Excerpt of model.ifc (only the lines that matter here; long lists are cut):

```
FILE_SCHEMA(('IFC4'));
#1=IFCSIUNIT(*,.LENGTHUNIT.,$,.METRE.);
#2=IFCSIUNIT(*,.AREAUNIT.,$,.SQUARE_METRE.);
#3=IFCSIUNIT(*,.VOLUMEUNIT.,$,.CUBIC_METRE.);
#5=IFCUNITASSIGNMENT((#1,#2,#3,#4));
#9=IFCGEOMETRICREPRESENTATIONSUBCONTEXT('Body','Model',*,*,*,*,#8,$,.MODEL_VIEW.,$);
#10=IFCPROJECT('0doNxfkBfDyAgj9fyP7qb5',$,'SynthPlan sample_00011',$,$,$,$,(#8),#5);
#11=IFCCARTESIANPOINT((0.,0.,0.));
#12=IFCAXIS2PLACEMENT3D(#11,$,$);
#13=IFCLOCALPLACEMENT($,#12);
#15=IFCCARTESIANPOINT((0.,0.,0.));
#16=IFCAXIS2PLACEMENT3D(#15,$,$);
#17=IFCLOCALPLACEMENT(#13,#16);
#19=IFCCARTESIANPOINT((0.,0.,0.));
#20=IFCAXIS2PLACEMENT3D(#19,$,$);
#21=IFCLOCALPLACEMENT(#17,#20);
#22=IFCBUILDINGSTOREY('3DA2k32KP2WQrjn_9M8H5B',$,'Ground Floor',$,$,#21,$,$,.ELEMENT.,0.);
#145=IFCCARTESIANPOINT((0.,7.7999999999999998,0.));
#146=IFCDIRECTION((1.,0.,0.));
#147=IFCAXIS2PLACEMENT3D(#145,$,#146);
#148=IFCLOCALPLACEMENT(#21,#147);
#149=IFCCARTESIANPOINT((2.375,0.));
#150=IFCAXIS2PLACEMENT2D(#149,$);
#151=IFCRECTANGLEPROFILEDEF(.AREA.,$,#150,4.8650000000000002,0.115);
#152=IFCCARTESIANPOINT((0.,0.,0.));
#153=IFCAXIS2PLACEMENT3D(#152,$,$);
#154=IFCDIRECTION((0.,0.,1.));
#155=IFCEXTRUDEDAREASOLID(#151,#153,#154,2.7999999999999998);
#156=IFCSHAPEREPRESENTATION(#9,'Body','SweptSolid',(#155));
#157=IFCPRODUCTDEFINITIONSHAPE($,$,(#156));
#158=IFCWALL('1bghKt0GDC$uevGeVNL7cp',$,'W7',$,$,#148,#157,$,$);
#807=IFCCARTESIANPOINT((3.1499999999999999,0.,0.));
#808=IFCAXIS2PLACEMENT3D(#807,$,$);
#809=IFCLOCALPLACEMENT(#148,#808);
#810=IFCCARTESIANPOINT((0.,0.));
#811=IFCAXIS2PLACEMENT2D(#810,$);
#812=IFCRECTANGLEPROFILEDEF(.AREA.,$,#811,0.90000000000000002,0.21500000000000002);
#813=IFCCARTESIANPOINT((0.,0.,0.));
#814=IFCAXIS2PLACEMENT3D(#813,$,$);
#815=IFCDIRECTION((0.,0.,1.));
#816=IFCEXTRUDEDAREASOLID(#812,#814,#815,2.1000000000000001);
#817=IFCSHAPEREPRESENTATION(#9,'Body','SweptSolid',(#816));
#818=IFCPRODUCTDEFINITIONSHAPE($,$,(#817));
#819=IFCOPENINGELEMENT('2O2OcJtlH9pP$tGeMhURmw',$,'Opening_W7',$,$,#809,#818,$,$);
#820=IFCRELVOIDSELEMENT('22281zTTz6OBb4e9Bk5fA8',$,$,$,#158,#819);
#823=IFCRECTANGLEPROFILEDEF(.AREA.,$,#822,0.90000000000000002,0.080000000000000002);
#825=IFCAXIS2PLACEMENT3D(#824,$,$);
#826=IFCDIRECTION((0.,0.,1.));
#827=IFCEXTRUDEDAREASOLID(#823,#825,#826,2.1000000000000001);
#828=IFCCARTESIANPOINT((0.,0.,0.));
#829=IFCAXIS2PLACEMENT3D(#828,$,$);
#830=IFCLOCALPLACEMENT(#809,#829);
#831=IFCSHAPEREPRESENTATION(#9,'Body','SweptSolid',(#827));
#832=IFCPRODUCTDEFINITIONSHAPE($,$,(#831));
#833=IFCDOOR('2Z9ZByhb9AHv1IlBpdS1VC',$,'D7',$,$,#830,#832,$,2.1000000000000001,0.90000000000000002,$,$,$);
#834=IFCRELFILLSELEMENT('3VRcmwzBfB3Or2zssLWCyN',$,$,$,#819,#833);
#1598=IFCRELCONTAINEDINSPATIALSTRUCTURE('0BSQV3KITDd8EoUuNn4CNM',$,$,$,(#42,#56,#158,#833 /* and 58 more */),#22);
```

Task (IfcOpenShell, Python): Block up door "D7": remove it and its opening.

```python
import ifcopenshell
import ifcopenshell.api.feature
import ifcopenshell.api.root
import ifcopenshell.geom
import ifcopenshell.util.shape

model = ifcopenshell.open("model.ifc")
settings = ifcopenshell.geom.settings()


def volume(element):
    """Net volume in cubic metres, openings subtracted."""
    shape = ifcopenshell.geom.create_shape(settings, element)
    return ifcopenshell.util.shape.get_volume(shape.geometry)


door = model.by_guid("2Z9ZByhb9AHv1IlBpdS1VC")
opening = door.FillsVoids[0].RelatingOpeningElement
wall = opening.VoidsElements[0].RelatingBuildingElement
before = volume(wall)

ifcopenshell.api.root.remove_product(model, product=door)
ifcopenshell.api.feature.remove_feature(model, feature=opening)

after = volume(wall)

print(f"wall volume {before:.3f} -> {after:.3f} m3")

model.write("model_rev.ifc")
```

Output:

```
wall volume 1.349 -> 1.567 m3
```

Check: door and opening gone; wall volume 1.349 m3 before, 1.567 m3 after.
